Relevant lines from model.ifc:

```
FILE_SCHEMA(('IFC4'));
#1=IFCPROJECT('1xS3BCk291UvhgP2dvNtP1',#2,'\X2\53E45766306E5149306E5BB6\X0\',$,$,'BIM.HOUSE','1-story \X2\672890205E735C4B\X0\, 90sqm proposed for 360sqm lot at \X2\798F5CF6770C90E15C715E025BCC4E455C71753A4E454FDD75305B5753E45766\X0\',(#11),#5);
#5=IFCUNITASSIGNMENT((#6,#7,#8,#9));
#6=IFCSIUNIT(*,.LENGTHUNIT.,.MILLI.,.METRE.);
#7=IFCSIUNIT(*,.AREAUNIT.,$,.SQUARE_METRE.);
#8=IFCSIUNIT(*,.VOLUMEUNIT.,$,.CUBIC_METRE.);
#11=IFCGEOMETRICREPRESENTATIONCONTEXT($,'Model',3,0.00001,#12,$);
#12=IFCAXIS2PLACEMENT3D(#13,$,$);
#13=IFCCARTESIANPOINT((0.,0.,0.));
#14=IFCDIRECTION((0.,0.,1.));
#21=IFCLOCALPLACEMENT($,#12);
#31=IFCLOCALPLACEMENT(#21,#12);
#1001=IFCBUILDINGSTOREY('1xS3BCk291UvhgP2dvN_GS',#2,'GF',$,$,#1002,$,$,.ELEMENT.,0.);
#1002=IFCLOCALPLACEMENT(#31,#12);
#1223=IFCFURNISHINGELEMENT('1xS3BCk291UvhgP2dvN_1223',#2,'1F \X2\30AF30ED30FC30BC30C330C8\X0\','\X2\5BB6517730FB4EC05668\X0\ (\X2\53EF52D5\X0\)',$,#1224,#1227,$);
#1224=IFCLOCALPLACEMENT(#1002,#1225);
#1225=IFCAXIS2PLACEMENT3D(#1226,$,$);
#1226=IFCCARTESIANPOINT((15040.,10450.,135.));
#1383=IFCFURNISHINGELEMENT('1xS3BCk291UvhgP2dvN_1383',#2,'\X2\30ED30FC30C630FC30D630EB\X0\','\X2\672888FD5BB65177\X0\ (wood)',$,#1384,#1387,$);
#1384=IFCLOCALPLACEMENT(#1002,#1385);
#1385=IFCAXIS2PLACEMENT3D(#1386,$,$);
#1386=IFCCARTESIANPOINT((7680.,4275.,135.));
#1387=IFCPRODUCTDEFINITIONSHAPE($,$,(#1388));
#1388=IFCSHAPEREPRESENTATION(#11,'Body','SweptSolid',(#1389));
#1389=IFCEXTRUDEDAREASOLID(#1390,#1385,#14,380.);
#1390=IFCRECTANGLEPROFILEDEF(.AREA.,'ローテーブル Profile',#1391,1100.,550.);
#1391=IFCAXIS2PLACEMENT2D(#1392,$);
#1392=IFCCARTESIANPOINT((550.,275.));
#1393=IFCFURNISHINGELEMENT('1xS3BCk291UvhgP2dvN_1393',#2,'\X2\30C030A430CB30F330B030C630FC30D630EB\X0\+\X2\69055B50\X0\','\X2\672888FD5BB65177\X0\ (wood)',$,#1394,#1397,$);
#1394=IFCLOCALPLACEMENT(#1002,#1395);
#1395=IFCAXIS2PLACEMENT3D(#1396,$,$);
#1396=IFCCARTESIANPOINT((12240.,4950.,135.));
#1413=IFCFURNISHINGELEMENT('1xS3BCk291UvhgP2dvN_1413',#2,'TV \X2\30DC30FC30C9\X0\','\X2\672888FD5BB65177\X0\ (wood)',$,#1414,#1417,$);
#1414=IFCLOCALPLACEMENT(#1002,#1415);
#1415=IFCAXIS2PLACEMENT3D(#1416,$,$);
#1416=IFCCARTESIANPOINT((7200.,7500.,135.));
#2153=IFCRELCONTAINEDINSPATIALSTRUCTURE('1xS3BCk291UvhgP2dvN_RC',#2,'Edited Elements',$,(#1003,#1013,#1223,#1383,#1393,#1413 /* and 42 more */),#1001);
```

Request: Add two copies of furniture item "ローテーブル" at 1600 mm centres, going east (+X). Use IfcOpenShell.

```python
import numpy as np
import ifcopenshell
import ifcopenshell.api.geometry
import ifcopenshell.api.root
import ifcopenshell.util.element
import ifcopenshell.util.placement
import ifcopenshell.util.unit

model = ifcopenshell.open("model.ifc")
unit_scale = ifcopenshell.util.unit.calculate_unit_scale(model)


def reuse_history(source, copy):
    """copy_class also copies each property set's owner history, people and application; keep the originals."""
    for rel in copy.IsDefinedBy:
        if rel.is_a("IfcRelDefinesByProperties") and (history := rel.RelatingPropertyDefinition.OwnerHistory):
            rel.RelatingPropertyDefinition.OwnerHistory = source.OwnerHistory
            ifcopenshell.util.element.remove_deep2(model, history)


source = model.by_id(1383)
base = ifcopenshell.util.placement.get_local_placement(source.ObjectPlacement)
step = np.array([1.0, 0.0, 0.0]) * 1.6 / unit_scale

for i in range(1, 3):
    copy = ifcopenshell.api.root.copy_class(model, product=source)
    copy.Representation = ifcopenshell.util.element.copy_deep(
        model, source.Representation, exclude=["IfcGeometricRepresentationContext", "IfcRepresentationMap"]
    )
    reuse_history(source, copy)
    matrix = base.copy()
    matrix[:3, 3] += i * step
    print("added at", matrix[:3, 3].round(3) + 0.0)
    ifcopenshell.api.geometry.edit_object_placement(model, product=copy, matrix=matrix, is_si=False)

model.write("model_updated.ifc")
```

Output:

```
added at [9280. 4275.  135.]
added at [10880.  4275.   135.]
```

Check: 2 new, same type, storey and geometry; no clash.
